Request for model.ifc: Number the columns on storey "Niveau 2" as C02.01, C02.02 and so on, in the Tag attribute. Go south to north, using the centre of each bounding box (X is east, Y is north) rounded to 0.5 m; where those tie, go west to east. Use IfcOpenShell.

First a look at what the model holds.

```python
import ifcopenshell
import ifcopenshell.util.element
import ifcopenshell.util.placement

model = ifcopenshell.open("model.ifc")
print(model.schema)
storey = next(s for s in model.by_type("IfcBuildingStorey") if s.Name == "Niveau 2")
columns = [e for e in ifcopenshell.util.element.get_decomposition(storey) if e.is_a("IfcColumn")]
for e in sorted(columns, key=lambda e: e.id()):
    origin = ifcopenshell.util.placement.get_local_placement(e.ObjectPlacement)[:3, 3]
    print(e.id(), e.Tag, e.Name, origin.round(2) + 0.0, sep=" | ")
```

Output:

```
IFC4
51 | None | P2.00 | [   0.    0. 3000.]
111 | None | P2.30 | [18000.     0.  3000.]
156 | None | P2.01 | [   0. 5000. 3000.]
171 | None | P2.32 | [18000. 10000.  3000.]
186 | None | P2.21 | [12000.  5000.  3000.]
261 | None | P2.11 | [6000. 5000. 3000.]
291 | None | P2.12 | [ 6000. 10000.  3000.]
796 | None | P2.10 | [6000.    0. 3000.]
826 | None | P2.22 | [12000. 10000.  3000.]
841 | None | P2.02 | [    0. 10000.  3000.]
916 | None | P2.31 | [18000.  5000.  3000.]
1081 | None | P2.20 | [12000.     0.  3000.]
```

```python
import ifcopenshell
import ifcopenshell.geom
import ifcopenshell.util.element
import ifcopenshell.util.shape

model = ifcopenshell.open("model.ifc")
settings = ifcopenshell.geom.settings()
settings.set("use-world-coords", True)


def centre(element):
    shape = ifcopenshell.geom.create_shape(settings, element)
    return ifcopenshell.util.shape.get_bbox_centroid(shape.geometry)


storey = next(s for s in model.by_type("IfcBuildingStorey") if s.Name == "Niveau 2")
columns = [e for e in ifcopenshell.util.element.get_decomposition(storey) if e.is_a("IfcColumn")]

# Insertion points can sit at a corner or the storey origin, so sort by the geometry (in metres).
centres = {e: centre(e) for e in columns}
columns.sort(key=lambda e: (round(centres[e][1] / 0.5), centres[e][0]))

for i, e in enumerate(columns, start=1):
    number = f"C02.{i:02d}"
    e.Tag = number
    print(e.id(), number)

model.write("model_updated.ifc")
```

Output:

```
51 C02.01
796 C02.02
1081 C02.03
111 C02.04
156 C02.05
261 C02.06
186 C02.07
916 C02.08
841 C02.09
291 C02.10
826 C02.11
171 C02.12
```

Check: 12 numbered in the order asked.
